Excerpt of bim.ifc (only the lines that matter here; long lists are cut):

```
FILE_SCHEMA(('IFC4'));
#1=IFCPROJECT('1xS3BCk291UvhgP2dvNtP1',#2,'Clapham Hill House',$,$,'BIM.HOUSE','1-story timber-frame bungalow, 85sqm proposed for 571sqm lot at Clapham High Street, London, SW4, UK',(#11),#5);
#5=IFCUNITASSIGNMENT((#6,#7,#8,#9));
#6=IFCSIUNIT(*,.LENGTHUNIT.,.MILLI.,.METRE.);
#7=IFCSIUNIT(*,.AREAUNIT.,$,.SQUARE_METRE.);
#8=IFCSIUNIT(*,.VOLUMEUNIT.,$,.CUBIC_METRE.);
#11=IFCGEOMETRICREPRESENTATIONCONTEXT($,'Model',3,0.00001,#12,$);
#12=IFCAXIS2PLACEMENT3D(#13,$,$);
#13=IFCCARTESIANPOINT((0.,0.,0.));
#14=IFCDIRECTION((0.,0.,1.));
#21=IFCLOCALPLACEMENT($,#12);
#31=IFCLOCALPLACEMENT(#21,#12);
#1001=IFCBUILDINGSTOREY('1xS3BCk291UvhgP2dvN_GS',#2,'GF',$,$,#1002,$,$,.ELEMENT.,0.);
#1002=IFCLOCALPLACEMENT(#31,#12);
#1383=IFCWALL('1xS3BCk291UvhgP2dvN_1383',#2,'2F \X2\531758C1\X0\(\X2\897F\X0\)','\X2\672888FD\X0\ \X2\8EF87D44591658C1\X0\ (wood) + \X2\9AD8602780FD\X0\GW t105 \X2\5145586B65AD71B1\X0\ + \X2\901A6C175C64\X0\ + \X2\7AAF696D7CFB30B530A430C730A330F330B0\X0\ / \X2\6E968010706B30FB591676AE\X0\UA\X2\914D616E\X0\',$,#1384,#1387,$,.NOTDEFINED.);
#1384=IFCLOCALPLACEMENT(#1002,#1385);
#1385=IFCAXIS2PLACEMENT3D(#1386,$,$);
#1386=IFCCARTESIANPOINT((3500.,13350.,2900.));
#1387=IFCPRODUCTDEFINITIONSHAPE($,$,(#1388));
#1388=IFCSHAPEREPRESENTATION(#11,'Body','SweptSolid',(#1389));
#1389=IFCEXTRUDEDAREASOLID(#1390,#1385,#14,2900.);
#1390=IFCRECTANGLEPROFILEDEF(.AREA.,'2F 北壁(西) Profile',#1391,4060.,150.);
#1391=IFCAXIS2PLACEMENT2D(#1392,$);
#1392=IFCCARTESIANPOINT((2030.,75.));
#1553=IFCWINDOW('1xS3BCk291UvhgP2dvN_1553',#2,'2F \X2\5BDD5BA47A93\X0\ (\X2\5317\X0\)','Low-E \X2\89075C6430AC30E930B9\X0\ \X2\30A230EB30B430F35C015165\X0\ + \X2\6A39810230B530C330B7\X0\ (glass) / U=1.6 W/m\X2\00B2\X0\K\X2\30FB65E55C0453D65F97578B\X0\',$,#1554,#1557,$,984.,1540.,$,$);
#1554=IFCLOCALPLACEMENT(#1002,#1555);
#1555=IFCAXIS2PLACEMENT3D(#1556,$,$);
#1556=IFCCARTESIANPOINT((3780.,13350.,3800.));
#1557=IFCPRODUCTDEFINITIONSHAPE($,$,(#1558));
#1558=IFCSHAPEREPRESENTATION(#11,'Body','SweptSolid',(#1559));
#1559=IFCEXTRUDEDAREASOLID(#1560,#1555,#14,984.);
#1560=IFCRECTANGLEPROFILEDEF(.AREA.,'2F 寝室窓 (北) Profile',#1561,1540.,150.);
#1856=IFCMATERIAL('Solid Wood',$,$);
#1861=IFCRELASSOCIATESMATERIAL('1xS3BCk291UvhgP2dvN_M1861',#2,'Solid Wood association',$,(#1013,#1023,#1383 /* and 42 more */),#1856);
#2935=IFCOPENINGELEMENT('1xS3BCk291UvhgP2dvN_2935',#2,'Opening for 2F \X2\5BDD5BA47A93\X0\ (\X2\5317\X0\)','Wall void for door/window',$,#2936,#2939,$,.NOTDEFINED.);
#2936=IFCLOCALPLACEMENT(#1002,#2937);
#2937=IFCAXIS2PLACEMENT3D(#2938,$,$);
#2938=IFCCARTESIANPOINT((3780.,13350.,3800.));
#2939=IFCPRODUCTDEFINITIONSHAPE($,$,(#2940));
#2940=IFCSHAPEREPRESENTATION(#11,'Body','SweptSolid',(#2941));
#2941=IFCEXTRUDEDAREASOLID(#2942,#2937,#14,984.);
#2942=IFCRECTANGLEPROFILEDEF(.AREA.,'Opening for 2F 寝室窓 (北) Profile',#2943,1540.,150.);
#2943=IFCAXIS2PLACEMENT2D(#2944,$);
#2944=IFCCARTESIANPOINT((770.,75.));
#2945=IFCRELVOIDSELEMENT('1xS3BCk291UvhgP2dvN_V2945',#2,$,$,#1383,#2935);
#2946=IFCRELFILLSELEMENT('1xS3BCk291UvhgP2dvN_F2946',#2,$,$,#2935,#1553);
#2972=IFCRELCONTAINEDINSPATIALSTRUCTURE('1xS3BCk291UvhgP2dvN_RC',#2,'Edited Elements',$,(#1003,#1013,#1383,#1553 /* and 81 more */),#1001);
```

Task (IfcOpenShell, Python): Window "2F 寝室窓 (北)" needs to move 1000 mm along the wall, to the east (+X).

```python
import ifcopenshell
import ifcopenshell.api.geometry
import ifcopenshell.util.placement
import ifcopenshell.util.unit

model = ifcopenshell.open("bim.ifc")
unit_scale = ifcopenshell.util.unit.calculate_unit_scale(model)

window = model.by_id(1553)
opening = window.FillsVoids[0].RelatingOpeningElement
wall = opening.VoidsElements[0].RelatingBuildingElement

wall_matrix = ifcopenshell.util.placement.get_local_placement(wall.ObjectPlacement)
shift = wall_matrix[:3, 0] * 1 / unit_scale
before = ifcopenshell.util.placement.get_local_placement(window.ObjectPlacement)[:3, 3].copy()

# The window is not placed relative to its opening, so move both.
for product in (opening, window):
    matrix = ifcopenshell.util.placement.get_local_placement(product.ObjectPlacement)
    matrix[:3, 3] += shift
    ifcopenshell.api.geometry.edit_object_placement(model, product=product, matrix=matrix, is_si=False)

after = ifcopenshell.util.placement.get_local_placement(window.ObjectPlacement)[:3, 3]
print("window moved by", (after - before).round(3) + 0.0)

model.write("bim_v2.ifc")
```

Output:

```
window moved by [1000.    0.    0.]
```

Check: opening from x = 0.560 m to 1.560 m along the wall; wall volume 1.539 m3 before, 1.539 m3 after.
